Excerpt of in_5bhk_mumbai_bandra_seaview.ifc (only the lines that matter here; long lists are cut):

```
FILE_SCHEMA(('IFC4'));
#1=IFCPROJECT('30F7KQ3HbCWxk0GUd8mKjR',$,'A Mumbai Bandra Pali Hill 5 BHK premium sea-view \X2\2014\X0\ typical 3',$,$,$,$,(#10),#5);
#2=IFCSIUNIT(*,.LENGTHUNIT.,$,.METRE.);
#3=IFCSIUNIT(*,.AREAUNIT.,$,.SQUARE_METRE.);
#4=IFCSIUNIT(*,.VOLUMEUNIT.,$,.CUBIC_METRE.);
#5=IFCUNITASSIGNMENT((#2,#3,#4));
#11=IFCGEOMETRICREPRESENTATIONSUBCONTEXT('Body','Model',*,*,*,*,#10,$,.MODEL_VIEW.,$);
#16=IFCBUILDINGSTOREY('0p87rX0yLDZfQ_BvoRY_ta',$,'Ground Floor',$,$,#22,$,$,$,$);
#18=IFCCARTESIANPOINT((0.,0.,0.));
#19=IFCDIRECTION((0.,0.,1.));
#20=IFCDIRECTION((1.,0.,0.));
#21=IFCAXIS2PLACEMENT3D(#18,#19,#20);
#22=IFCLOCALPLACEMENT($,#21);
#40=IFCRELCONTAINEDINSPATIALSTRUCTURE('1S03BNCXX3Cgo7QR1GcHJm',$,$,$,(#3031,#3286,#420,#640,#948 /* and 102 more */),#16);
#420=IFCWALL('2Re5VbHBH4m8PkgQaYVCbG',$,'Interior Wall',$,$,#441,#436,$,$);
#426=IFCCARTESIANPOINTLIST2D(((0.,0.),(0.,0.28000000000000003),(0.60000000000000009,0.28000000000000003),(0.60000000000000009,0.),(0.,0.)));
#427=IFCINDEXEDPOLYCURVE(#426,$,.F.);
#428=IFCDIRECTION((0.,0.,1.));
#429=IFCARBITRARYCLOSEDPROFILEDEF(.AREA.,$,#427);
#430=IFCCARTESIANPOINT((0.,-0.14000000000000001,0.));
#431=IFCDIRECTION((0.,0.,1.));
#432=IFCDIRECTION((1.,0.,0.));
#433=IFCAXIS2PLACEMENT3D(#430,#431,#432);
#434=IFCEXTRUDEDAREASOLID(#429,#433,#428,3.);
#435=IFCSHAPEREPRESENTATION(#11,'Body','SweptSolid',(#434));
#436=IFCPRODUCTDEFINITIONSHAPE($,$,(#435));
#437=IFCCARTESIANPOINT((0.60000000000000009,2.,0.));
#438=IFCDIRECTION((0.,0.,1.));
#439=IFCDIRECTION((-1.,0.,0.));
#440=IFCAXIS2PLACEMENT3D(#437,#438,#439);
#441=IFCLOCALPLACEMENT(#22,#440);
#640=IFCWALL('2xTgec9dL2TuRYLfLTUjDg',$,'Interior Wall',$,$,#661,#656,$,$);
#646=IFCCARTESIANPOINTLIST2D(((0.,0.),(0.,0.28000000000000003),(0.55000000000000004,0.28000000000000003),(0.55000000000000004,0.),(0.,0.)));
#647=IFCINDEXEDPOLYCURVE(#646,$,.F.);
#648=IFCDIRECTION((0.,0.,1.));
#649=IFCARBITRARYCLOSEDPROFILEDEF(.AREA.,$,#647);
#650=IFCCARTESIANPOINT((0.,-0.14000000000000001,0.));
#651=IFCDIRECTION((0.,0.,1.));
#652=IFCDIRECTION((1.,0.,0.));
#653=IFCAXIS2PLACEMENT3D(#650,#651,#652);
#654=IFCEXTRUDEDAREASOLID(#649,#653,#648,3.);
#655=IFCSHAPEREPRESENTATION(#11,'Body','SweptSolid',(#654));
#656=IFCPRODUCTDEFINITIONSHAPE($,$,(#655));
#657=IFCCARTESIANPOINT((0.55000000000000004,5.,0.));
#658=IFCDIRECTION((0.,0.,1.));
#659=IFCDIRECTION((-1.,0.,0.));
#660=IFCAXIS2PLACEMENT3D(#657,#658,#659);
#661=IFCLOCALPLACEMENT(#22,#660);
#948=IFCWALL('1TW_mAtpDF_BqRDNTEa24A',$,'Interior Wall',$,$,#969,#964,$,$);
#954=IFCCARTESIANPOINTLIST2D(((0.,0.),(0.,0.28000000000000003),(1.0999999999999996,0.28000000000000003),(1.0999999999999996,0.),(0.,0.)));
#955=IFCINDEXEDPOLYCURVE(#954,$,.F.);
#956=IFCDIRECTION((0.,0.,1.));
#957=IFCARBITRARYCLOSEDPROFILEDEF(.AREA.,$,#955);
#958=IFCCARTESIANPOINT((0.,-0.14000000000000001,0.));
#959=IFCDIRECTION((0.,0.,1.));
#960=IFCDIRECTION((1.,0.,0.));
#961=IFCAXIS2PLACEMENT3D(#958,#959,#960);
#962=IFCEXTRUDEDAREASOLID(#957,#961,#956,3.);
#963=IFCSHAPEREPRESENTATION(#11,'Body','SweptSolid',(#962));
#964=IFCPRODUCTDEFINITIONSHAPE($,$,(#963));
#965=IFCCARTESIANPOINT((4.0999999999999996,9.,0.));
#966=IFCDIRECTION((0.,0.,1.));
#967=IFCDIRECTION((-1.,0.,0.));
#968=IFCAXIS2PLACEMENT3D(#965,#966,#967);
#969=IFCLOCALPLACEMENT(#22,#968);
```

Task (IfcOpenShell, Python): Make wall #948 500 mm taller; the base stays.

```python
import ifcopenshell
import ifcopenshell.geom
import ifcopenshell.util.representation
import ifcopenshell.util.shape

model = ifcopenshell.open("in_5bhk_mumbai_bandra_seaview.ifc")
settings = ifcopenshell.geom.settings()


def volume(element):
    """Net volume in cubic metres, openings subtracted."""
    shape = ifcopenshell.geom.create_shape(settings, element)
    return ifcopenshell.util.shape.get_volume(shape.geometry)


wall = model.by_guid("1TW_mAtpDF_BqRDNTEa24A")
before = volume(wall)

body = ifcopenshell.util.representation.get_representation(wall, "Model", "Body")
solid = body.Items[0]
old_height = solid.Depth
solid.Depth += 0.5
after = volume(wall)

print(f"height {old_height:g} -> {solid.Depth:g}, volume {before:.3f} -> {after:.3f} m3")

model.write("in_5bhk_mumbai_bandra_seaview-out.ifc")
```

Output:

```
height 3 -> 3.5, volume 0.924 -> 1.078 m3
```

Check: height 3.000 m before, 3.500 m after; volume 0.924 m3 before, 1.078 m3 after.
